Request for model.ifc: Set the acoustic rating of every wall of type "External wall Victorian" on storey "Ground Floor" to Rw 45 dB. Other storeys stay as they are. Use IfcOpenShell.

First a look at what the model holds.

```python
import ifcopenshell
import ifcopenshell.util.element

model = ifcopenshell.open("model.ifc")
print(model.schema)
storey = next(s for s in model.by_type("IfcBuildingStorey") if s.Name == "Ground Floor")
walls = [e for e in ifcopenshell.util.element.get_decomposition(storey) if e.is_a("IfcWall")]
seen = {}
for e in walls:
    element_type = ifcopenshell.util.element.get_type(e)
    key = (element_type.Name if element_type != e and element_type else None, ifcopenshell.util.element.get_pset(e, "Pset_WallCommon", "AcousticRating"))
    seen[key] = seen.get(key, 0) + 1
for (name, value), count in sorted(seen.items(), key=str):
    print(count, "x", name, "|", value)
```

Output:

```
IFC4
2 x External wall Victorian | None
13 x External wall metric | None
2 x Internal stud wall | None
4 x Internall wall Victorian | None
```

```python
import ifcopenshell
import ifcopenshell.api.pset
import ifcopenshell.util.element

model = ifcopenshell.open("model.ifc")

storey = next(s for s in model.by_type("IfcBuildingStorey") if s.Name == "Ground Floor")
walls = [e for e in ifcopenshell.util.element.get_decomposition(storey) if e.is_a("IfcWall")]

count = 0
for e in walls:
    element_type = ifcopenshell.util.element.get_type(e)
    if element_type in (None, e) or element_type.Name != "External wall Victorian":
        continue
    # add_pset returns the element's existing set when there is one.
    pset = ifcopenshell.api.pset.add_pset(model, product=e, name="Pset_WallCommon")
    ifcopenshell.api.pset.edit_pset(model, pset=pset, properties={"AcousticRating": "Rw 45 dB"})
    count += 1

print(count, "walls updated")

model.write("model_rev.ifc")
```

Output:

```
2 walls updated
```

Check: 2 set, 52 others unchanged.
